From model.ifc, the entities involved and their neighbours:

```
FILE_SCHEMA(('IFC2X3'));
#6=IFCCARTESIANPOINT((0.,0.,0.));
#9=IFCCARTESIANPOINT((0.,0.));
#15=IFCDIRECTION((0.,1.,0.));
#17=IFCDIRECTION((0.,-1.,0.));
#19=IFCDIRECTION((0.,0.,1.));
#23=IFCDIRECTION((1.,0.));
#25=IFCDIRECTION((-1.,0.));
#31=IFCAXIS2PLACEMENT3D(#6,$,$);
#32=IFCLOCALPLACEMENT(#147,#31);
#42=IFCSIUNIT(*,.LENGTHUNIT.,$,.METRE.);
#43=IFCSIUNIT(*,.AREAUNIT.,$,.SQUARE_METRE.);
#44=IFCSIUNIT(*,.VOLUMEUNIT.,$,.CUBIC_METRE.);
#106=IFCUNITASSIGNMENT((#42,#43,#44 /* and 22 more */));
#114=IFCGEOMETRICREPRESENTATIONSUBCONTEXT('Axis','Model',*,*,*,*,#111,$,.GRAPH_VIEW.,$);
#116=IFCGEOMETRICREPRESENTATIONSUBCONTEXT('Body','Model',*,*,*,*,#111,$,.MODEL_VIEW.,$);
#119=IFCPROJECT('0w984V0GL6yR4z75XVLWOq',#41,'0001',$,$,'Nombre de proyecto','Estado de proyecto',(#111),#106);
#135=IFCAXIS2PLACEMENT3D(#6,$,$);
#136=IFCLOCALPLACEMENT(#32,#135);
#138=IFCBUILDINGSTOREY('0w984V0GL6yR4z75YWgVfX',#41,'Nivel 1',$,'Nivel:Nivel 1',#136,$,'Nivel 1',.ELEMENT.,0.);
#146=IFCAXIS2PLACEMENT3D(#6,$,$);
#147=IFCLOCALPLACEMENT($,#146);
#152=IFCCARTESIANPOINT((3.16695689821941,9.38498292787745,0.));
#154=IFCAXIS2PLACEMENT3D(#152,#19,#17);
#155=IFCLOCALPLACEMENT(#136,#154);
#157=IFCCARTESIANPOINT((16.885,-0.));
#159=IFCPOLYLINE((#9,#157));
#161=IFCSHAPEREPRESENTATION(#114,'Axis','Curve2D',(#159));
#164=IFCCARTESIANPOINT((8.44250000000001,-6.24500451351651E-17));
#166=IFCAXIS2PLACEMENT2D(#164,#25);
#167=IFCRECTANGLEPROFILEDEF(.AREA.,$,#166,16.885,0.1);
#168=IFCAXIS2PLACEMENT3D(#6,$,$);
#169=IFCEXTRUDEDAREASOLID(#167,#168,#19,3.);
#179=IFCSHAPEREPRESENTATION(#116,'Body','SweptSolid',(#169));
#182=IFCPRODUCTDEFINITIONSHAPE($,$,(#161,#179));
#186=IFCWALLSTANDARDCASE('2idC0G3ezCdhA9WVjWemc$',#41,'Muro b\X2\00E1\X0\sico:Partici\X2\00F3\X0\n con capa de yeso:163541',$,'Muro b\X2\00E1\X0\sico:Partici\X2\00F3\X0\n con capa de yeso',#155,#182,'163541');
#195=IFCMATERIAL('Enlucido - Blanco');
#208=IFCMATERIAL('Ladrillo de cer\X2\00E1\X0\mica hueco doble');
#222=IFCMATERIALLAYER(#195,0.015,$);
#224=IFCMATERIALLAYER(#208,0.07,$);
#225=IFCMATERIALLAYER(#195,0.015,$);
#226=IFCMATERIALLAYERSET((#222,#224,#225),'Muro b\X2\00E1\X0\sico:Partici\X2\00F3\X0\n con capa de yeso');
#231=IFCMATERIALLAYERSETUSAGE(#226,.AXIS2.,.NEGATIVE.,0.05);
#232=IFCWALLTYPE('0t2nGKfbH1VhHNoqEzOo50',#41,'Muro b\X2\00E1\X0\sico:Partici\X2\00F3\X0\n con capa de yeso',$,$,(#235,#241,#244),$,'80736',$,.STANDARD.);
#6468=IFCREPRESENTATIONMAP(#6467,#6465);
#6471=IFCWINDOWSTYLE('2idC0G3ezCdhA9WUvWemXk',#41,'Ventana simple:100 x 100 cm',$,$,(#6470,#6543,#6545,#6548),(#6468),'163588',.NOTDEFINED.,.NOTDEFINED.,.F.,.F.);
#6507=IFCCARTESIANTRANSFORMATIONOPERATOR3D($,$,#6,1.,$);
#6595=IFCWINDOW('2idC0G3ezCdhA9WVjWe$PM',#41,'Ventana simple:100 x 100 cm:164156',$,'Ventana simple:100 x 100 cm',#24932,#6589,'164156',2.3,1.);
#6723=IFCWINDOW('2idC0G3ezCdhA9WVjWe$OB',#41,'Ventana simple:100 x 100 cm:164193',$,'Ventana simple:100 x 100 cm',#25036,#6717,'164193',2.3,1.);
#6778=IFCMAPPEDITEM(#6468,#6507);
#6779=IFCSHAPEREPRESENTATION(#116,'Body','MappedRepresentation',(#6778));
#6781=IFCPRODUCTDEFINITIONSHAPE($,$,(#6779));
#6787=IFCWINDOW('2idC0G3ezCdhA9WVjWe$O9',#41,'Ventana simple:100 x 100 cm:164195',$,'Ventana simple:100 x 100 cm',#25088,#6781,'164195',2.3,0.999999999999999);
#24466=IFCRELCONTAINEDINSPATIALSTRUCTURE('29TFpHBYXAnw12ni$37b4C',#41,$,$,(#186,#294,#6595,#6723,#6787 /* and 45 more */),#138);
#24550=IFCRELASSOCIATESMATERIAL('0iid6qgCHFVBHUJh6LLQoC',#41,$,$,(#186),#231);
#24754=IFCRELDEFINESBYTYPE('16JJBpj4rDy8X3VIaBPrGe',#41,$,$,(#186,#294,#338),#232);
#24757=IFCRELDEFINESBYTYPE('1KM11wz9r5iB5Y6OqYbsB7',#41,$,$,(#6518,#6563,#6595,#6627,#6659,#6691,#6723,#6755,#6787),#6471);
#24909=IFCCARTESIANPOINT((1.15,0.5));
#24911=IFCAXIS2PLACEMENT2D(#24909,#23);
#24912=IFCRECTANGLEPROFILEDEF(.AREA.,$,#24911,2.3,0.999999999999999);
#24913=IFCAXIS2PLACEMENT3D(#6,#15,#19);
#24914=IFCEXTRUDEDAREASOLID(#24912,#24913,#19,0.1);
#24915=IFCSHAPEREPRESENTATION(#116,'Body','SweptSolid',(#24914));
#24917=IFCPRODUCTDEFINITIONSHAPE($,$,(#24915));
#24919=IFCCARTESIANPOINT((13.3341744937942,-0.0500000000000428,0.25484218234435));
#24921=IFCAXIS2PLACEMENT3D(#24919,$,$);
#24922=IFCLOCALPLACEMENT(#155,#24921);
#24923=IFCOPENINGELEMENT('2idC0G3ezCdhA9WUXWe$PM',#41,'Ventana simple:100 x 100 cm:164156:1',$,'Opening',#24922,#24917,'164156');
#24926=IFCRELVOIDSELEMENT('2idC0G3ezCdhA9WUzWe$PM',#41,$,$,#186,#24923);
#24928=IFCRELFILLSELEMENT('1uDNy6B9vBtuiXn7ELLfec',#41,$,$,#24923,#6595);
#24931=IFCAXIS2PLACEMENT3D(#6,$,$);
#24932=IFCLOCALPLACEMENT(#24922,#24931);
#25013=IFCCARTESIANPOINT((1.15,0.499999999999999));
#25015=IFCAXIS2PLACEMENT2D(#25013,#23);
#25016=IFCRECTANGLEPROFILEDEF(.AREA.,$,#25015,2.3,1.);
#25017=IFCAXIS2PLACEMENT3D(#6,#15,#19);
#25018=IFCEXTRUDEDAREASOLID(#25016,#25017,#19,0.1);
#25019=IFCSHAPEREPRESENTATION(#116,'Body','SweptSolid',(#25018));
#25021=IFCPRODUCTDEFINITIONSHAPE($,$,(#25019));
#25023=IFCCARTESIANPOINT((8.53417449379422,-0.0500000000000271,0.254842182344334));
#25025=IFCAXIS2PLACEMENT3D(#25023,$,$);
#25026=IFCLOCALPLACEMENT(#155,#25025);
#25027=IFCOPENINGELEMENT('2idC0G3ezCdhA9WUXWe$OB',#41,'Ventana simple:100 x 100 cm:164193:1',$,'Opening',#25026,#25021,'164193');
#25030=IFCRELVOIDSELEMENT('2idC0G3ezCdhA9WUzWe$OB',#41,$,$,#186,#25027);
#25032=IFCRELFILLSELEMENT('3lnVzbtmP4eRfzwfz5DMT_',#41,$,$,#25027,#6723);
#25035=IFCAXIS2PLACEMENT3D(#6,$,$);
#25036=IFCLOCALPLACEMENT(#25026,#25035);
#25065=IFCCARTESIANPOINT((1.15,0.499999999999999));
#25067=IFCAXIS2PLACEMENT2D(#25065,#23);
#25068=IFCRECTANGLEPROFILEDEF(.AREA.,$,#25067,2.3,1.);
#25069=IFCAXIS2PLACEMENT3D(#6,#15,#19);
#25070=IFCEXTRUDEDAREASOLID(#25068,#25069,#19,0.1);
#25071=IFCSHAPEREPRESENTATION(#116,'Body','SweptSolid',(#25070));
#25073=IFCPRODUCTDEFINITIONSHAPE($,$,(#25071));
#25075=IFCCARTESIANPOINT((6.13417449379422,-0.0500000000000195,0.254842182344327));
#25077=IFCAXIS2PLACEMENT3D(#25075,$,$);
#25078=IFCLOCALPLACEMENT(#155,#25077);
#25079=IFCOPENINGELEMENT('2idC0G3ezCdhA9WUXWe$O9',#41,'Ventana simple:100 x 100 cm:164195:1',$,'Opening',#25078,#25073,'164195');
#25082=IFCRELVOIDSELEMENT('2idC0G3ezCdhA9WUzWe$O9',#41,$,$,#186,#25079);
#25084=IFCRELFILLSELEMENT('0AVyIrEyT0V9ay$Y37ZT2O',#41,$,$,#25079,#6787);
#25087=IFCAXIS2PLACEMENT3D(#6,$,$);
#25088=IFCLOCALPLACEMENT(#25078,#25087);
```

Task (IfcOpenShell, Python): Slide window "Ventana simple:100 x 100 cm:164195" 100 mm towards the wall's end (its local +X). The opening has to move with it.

```python
import ifcopenshell
import ifcopenshell.api.geometry
import ifcopenshell.util.placement

model = ifcopenshell.open("model.ifc")

window = model.by_guid("2idC0G3ezCdhA9WVjWe$O9")
opening = window.FillsVoids[0].RelatingOpeningElement
wall = opening.VoidsElements[0].RelatingBuildingElement

wall_matrix = ifcopenshell.util.placement.get_local_placement(wall.ObjectPlacement)
shift = wall_matrix[:3, 0] * 0.1
before = ifcopenshell.util.placement.get_local_placement(window.ObjectPlacement)[:3, 3].copy()

# The window is placed relative to its opening, so it follows when the opening moves.
matrix = ifcopenshell.util.placement.get_local_placement(opening.ObjectPlacement)
matrix[:3, 3] += shift
ifcopenshell.api.geometry.edit_object_placement(
    model, product=opening, matrix=matrix, is_si=False, should_transform_children=True
)

after = ifcopenshell.util.placement.get_local_placement(window.ObjectPlacement)[:3, 3]
print("window moved by", (after - before).round(3) + 0.0)

model.write("model_rev.ifc")
```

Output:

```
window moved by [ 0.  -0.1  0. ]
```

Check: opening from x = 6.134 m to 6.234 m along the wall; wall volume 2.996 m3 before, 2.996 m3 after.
